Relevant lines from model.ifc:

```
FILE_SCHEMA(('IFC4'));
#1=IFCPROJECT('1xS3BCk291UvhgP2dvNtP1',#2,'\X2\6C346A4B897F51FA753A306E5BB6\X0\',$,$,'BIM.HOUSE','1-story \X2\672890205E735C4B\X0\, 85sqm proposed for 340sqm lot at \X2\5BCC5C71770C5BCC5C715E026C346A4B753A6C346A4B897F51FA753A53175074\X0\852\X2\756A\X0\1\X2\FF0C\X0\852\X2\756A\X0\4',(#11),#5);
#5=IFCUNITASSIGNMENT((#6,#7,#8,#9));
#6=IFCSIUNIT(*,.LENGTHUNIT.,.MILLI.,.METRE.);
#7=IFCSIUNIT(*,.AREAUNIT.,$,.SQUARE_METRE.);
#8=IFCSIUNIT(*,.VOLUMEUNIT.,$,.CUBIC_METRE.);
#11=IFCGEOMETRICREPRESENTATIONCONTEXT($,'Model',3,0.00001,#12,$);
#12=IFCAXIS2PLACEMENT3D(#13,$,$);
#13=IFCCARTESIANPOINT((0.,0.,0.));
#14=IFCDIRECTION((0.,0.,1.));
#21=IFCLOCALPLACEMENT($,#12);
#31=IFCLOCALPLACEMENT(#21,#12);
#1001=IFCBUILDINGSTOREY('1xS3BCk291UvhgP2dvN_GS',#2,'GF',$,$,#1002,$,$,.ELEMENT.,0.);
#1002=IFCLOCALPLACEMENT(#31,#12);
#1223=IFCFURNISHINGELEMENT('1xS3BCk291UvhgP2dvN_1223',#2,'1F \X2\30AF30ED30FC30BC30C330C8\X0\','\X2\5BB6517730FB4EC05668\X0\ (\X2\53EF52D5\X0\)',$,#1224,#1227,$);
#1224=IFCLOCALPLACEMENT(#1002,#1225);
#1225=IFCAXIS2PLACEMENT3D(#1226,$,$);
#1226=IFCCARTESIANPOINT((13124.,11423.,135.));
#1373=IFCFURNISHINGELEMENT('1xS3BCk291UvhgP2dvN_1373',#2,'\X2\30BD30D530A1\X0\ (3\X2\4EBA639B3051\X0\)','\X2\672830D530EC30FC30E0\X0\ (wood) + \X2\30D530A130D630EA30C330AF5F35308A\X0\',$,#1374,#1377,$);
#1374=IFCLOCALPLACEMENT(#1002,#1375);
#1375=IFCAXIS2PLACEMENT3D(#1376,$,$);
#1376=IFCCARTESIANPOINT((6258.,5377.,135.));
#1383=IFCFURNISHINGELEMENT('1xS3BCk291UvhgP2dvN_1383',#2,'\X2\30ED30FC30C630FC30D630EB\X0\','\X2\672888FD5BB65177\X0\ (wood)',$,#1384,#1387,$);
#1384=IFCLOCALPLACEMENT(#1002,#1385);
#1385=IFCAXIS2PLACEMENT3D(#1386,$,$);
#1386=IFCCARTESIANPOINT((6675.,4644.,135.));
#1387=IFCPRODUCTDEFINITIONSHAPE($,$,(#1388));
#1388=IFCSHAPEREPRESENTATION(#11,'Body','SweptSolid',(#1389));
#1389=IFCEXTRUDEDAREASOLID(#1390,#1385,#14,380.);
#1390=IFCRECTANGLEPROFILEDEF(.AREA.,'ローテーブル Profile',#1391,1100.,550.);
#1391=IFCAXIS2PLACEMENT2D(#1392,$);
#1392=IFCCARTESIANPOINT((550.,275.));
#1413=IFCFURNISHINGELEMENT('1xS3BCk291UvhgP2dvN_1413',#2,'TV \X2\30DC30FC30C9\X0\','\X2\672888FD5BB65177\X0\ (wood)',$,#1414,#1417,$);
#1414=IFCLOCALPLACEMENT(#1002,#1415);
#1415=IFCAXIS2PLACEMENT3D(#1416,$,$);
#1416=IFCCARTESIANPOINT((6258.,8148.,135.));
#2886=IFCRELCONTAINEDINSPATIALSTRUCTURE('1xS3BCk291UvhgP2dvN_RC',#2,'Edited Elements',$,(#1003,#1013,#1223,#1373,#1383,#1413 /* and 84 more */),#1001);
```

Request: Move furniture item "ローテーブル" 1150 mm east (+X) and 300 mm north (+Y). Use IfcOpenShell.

```python
import ifcopenshell
import ifcopenshell.api.geometry
import ifcopenshell.util.placement

model = ifcopenshell.open("model.ifc")

item = model.by_guid("1xS3BCk291UvhgP2dvN_1383")
matrix = ifcopenshell.util.placement.get_local_placement(item.ObjectPlacement)
matrix[0, 3] += 1150.0
matrix[1, 3] += 300.0
ifcopenshell.api.geometry.edit_object_placement(model, product=item, matrix=matrix, is_si=False)

print(ifcopenshell.util.placement.get_local_placement(item.ObjectPlacement).round(3) + 0.0)

model.write("model_edited.ifc")
```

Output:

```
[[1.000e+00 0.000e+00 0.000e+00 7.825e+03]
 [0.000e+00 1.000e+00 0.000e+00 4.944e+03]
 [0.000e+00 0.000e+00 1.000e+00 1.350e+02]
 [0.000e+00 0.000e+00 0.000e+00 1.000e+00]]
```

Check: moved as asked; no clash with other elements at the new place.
